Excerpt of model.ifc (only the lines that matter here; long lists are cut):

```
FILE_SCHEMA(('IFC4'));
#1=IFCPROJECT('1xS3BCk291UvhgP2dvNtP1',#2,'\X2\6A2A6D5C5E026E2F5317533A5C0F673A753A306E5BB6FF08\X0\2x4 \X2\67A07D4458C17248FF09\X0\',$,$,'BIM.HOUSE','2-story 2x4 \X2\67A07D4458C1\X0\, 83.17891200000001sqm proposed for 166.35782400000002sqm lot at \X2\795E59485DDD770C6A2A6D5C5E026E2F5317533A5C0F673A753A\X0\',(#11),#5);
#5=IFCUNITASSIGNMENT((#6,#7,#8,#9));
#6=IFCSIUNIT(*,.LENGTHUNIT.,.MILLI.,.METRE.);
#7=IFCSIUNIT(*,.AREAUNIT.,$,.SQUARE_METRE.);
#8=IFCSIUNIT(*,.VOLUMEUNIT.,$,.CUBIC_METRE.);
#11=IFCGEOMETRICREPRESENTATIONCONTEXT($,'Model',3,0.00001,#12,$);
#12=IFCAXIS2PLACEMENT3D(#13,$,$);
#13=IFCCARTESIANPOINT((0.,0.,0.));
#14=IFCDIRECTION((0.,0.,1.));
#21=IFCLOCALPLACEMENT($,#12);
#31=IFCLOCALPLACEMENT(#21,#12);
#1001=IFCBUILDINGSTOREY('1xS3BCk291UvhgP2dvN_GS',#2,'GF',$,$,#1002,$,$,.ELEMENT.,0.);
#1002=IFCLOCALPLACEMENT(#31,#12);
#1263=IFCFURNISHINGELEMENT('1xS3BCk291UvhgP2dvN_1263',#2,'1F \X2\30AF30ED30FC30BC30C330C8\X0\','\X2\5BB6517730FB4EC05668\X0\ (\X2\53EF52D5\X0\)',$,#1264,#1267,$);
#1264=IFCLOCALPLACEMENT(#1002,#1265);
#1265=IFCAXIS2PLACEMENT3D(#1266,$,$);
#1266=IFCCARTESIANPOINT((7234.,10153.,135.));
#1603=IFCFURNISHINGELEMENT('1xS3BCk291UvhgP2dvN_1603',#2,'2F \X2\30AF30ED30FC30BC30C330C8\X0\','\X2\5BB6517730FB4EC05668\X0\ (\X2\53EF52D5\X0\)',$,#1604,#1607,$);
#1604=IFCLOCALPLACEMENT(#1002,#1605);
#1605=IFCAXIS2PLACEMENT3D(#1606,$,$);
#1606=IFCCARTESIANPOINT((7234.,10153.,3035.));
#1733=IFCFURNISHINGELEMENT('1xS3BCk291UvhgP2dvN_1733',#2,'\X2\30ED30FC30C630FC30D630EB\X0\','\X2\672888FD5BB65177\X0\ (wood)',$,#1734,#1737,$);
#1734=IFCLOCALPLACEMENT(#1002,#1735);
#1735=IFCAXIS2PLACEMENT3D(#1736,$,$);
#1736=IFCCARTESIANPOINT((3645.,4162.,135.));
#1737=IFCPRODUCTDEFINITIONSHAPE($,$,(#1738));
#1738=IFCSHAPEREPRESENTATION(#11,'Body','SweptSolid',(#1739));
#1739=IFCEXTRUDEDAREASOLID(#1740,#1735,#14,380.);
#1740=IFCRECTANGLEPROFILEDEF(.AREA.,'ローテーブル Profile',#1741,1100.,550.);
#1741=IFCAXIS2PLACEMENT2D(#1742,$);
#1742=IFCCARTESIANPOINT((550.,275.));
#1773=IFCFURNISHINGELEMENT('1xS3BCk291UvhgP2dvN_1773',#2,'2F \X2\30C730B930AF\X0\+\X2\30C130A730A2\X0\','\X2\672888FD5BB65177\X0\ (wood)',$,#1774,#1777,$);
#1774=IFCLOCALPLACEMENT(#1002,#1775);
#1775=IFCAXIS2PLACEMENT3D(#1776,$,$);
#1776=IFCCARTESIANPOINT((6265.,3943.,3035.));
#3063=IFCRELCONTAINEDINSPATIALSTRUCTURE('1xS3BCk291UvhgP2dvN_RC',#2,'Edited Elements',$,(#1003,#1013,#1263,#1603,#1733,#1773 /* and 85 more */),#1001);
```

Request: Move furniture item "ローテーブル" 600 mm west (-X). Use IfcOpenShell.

```python
import ifcopenshell
import ifcopenshell.api.geometry
import ifcopenshell.util.placement
import ifcopenshell.util.unit

model = ifcopenshell.open("model.ifc")
unit_scale = ifcopenshell.util.unit.calculate_unit_scale(model)

item = model.by_guid("1xS3BCk291UvhgP2dvN_1733")
matrix = ifcopenshell.util.placement.get_local_placement(item.ObjectPlacement)
matrix[0, 3] -= 0.6 / unit_scale
ifcopenshell.api.geometry.edit_object_placement(model, product=item, matrix=matrix, is_si=False)

print(ifcopenshell.util.placement.get_local_placement(item.ObjectPlacement).round(3) + 0.0)

model.write("model_updated.ifc")
```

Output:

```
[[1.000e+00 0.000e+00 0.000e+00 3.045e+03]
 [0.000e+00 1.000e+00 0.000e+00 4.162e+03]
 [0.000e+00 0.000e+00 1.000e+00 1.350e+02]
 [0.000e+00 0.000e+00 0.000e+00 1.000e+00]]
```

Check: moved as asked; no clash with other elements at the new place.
